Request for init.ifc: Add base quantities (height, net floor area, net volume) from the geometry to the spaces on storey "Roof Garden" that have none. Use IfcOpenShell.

First a look at what the model holds.

```python
import ifcopenshell
import ifcopenshell.util.element
import ifcopenshell.util.unit

model = ifcopenshell.open("init.ifc")
print(model.schema)
for unit_type in ("LENGTHUNIT", "AREAUNIT", "VOLUMEUNIT"):
    print(unit_type, ifcopenshell.util.unit.calculate_unit_scale(model, unit_type))
storey = next(s for s in model.by_type("IfcBuildingStorey") if s.Name == "Roof Garden")
spaces = [e for e in ifcopenshell.util.element.get_decomposition(storey) if e.is_a("IfcSpace")]
for e in sorted(spaces, key=lambda e: e.id()):
    print(e.id(), e.is_a(), e.Name, list(ifcopenshell.util.element.get_psets(e, qtos_only=True)), sep=" | ")
```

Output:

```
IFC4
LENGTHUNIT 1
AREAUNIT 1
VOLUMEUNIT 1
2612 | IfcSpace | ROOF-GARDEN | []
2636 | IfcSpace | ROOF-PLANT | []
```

```python
import ifcopenshell
import ifcopenshell.api.pset
import ifcopenshell.geom
import ifcopenshell.util.element
import ifcopenshell.util.shape
import ifcopenshell.util.unit

model = ifcopenshell.open("init.ifc")
unit_scale = ifcopenshell.util.unit.calculate_unit_scale(model)
area_scale = ifcopenshell.util.unit.calculate_unit_scale(model, "AREAUNIT")
volume_scale = ifcopenshell.util.unit.calculate_unit_scale(model, "VOLUMEUNIT")
settings = ifcopenshell.geom.settings()

storey = next(s for s in model.by_type("IfcBuildingStorey") if s.Name == "Roof Garden")
spaces = [e for e in ifcopenshell.util.element.get_decomposition(storey) if e.is_a("IfcSpace")]

for e in sorted(spaces, key=lambda e: e.id()):
    if ifcopenshell.util.element.get_psets(e, qtos_only=True, should_inherit=False):
        continue
    # Geometry comes back in metres, in the element's own axes.
    shape = ifcopenshell.geom.create_shape(settings, e)
    values = {
        "Height": ifcopenshell.util.shape.get_z(shape.geometry) / unit_scale,
        "NetFloorArea": ifcopenshell.util.shape.get_footprint_area(shape.geometry) / area_scale,
        "NetVolume": ifcopenshell.util.shape.get_volume(shape.geometry) / volume_scale,
    }
    qto = ifcopenshell.api.pset.add_qto(model, product=e, name="Qto_SpaceBaseQuantities")
    ifcopenshell.api.pset.edit_qto(model, qto=qto, properties=values)
    print(e.id(), {k: round(v, 3) for k, v in values.items()})

model.write("init_updated.ifc")
```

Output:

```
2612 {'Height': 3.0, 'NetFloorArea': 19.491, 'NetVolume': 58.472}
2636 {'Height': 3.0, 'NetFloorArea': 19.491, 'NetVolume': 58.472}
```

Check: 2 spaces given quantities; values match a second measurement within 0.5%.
